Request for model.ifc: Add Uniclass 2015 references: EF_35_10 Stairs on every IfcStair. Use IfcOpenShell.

First a look at what the model holds.

```python
import ifcopenshell

model = ifcopenshell.open("model.ifc")
print(model.schema)
print("classifications:", [c.Name for c in model.by_type("IfcClassification")])
for ifc_class in ("IfcDoor", "IfcRoof", "IfcStair", "IfcWall", "IfcWindow"):
    print(ifc_class, len(model.by_type(ifc_class)))
```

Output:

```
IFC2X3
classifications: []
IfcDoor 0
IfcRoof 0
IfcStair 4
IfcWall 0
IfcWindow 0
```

```python
import ifcopenshell
import ifcopenshell.api.classification

model = ifcopenshell.open("model.ifc")

# IFC2X3 requires Source and Edition and has no link from the project to the system.
system = model.create_entity("IfcClassification", Source="NBS", Edition="2015", Name="Uniclass 2015")

codes = {
    "IfcStair": ("EF_35_10", "Stairs"),
}
for ifc_class, (code, name) in codes.items():
    products = model.by_type(ifc_class)
    ifcopenshell.api.classification.add_reference(
        model, products=products, classification=system, identification=code, name=name
    )
    print(code, len(products))

model.write("model_v2.ifc")
```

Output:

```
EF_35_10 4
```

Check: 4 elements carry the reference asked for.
